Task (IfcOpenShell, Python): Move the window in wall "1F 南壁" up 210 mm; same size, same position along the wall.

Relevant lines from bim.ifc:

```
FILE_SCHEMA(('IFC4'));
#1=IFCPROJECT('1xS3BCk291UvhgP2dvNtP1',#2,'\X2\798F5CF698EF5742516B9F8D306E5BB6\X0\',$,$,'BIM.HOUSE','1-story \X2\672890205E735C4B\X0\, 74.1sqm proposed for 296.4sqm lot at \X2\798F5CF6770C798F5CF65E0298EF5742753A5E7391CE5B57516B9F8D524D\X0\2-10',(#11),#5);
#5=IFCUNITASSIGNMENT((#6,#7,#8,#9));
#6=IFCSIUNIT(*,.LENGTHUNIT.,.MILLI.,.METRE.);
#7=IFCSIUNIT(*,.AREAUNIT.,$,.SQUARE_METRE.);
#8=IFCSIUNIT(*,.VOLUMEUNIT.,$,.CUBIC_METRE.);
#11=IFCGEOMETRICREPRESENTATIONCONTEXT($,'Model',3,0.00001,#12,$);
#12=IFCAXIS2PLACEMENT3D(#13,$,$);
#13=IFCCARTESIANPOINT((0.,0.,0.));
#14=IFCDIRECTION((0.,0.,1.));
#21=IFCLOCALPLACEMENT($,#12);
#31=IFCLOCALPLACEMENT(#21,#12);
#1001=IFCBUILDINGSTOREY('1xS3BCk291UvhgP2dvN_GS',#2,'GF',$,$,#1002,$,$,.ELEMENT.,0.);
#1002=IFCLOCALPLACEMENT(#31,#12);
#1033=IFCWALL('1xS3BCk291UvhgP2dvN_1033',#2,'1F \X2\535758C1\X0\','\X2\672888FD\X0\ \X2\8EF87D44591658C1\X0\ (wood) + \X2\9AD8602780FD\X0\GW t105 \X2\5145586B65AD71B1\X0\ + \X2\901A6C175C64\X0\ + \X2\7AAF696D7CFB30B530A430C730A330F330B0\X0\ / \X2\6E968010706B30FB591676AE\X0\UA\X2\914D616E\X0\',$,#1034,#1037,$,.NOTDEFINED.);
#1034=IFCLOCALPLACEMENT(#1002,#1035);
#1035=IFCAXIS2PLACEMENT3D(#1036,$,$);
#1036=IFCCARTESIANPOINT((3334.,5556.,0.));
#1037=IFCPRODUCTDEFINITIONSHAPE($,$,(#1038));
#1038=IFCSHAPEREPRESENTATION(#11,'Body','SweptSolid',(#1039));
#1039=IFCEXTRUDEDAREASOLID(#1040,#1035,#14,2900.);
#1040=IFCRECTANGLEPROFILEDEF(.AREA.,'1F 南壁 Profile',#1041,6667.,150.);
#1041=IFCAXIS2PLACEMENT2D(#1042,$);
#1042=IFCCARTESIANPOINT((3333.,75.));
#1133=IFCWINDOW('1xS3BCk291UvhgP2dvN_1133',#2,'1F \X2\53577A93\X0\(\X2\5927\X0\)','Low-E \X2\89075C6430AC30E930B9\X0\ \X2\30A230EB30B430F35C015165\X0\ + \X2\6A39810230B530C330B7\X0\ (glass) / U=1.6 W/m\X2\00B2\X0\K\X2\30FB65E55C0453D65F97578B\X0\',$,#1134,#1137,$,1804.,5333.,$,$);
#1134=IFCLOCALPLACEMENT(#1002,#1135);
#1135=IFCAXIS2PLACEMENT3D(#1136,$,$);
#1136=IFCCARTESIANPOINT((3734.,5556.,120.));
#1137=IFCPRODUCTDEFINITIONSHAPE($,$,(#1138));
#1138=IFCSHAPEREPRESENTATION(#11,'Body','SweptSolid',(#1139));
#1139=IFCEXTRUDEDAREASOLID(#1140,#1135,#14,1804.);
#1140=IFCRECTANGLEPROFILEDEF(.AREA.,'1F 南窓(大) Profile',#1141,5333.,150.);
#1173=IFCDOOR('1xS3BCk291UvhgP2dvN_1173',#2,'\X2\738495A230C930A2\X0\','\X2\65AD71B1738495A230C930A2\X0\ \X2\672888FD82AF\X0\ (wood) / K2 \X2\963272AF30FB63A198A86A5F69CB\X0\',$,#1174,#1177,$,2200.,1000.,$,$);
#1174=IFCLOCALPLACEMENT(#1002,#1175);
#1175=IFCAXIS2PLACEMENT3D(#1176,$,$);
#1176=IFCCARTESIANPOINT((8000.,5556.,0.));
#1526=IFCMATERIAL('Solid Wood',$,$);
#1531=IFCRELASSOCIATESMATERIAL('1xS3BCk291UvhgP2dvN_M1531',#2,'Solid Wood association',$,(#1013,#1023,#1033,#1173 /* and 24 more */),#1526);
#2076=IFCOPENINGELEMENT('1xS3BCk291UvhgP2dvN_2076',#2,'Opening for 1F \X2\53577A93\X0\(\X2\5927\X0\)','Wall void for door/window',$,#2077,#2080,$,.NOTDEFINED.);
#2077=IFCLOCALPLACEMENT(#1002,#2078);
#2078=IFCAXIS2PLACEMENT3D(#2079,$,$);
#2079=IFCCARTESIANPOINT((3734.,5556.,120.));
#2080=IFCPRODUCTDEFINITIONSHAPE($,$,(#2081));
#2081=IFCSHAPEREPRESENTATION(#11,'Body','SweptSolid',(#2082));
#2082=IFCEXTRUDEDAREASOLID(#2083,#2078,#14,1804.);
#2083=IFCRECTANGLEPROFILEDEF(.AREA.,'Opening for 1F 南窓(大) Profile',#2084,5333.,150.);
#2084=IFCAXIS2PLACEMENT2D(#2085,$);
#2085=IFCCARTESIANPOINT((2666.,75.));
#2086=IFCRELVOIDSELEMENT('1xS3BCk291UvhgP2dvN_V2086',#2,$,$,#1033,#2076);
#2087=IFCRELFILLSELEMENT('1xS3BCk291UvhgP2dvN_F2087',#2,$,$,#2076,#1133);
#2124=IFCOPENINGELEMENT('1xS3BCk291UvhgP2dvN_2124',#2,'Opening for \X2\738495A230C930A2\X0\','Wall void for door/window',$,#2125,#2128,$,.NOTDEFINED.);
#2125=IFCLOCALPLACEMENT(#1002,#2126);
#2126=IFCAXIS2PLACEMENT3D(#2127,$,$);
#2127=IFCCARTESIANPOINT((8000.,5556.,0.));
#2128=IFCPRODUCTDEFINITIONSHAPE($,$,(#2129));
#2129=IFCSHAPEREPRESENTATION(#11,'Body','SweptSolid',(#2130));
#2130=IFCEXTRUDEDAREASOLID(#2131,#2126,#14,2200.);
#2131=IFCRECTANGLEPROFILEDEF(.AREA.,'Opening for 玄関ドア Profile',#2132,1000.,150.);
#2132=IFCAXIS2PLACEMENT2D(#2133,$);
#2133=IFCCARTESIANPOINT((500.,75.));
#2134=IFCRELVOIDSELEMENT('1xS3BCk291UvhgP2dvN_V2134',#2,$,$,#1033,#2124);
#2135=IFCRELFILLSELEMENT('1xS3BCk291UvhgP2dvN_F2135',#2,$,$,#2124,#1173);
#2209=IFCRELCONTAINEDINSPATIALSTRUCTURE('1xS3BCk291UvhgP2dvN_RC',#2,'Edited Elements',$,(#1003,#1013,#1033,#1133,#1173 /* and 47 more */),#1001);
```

```python
import numpy as np
import ifcopenshell
import ifcopenshell.api.geometry
import ifcopenshell.util.placement
import ifcopenshell.util.unit

model = ifcopenshell.open("bim.ifc")
unit_scale = ifcopenshell.util.unit.calculate_unit_scale(model)

window = model.by_guid("1xS3BCk291UvhgP2dvN_1133")
opening = window.FillsVoids[0].RelatingOpeningElement
dz = 210.0

shift = np.array([0.0, 0.0, dz])
# The window is not placed relative to its opening, so move both.
for product in (opening, window):
    matrix = ifcopenshell.util.placement.get_local_placement(product.ObjectPlacement)
    matrix[:3, 3] += shift
    ifcopenshell.api.geometry.edit_object_placement(model, product=product, matrix=matrix, is_si=False)

print(f"moved by {dz * unit_scale:+.3f} m")

model.write("bim_updated.ifc")
```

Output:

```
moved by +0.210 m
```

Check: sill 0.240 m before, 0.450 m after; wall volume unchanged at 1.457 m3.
